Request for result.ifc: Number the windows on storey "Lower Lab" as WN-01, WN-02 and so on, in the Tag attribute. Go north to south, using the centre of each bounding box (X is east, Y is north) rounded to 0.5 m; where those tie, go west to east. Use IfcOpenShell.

First a look at what the model holds.

```python
import ifcopenshell
import ifcopenshell.util.element
import ifcopenshell.util.placement

model = ifcopenshell.open("result.ifc")
print(model.schema)
storey = next(s for s in model.by_type("IfcBuildingStorey") if s.Name == "Lower Lab")
windows = [e for e in ifcopenshell.util.element.get_decomposition(storey) if e.is_a("IfcWindow")]
for e in sorted(windows, key=lambda e: e.id()):
    origin = ifcopenshell.util.placement.get_local_placement(e.ObjectPlacement)[:3, 3]
    print(e.id(), e.Tag, e.Name, origin.round(2) + 0.0, sep=" | ")
```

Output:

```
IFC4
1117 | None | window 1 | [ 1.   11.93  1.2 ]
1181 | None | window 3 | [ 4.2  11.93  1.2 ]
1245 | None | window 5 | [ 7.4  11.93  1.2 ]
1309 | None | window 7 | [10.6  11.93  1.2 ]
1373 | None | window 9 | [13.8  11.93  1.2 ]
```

```python
import ifcopenshell
import ifcopenshell.geom
import ifcopenshell.util.element
import ifcopenshell.util.shape

model = ifcopenshell.open("result.ifc")
settings = ifcopenshell.geom.settings()
settings.set("use-world-coords", True)


def centre(element):
    shape = ifcopenshell.geom.create_shape(settings, element)
    return ifcopenshell.util.shape.get_bbox_centroid(shape.geometry)


storey = next(s for s in model.by_type("IfcBuildingStorey") if s.Name == "Lower Lab")
windows = [e for e in ifcopenshell.util.element.get_decomposition(storey) if e.is_a("IfcWindow")]

# Insertion points can sit at a corner or the storey origin, so sort by the geometry (in metres).
centres = {e: centre(e) for e in windows}
windows.sort(key=lambda e: (-round(centres[e][1] / 0.5), centres[e][0]))

for i, e in enumerate(windows, start=1):
    number = f"WN-{i:02d}"
    e.Tag = number
    print(e.id(), number)

model.write("result_updated.ifc")
```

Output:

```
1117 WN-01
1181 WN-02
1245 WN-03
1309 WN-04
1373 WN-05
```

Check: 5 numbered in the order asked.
